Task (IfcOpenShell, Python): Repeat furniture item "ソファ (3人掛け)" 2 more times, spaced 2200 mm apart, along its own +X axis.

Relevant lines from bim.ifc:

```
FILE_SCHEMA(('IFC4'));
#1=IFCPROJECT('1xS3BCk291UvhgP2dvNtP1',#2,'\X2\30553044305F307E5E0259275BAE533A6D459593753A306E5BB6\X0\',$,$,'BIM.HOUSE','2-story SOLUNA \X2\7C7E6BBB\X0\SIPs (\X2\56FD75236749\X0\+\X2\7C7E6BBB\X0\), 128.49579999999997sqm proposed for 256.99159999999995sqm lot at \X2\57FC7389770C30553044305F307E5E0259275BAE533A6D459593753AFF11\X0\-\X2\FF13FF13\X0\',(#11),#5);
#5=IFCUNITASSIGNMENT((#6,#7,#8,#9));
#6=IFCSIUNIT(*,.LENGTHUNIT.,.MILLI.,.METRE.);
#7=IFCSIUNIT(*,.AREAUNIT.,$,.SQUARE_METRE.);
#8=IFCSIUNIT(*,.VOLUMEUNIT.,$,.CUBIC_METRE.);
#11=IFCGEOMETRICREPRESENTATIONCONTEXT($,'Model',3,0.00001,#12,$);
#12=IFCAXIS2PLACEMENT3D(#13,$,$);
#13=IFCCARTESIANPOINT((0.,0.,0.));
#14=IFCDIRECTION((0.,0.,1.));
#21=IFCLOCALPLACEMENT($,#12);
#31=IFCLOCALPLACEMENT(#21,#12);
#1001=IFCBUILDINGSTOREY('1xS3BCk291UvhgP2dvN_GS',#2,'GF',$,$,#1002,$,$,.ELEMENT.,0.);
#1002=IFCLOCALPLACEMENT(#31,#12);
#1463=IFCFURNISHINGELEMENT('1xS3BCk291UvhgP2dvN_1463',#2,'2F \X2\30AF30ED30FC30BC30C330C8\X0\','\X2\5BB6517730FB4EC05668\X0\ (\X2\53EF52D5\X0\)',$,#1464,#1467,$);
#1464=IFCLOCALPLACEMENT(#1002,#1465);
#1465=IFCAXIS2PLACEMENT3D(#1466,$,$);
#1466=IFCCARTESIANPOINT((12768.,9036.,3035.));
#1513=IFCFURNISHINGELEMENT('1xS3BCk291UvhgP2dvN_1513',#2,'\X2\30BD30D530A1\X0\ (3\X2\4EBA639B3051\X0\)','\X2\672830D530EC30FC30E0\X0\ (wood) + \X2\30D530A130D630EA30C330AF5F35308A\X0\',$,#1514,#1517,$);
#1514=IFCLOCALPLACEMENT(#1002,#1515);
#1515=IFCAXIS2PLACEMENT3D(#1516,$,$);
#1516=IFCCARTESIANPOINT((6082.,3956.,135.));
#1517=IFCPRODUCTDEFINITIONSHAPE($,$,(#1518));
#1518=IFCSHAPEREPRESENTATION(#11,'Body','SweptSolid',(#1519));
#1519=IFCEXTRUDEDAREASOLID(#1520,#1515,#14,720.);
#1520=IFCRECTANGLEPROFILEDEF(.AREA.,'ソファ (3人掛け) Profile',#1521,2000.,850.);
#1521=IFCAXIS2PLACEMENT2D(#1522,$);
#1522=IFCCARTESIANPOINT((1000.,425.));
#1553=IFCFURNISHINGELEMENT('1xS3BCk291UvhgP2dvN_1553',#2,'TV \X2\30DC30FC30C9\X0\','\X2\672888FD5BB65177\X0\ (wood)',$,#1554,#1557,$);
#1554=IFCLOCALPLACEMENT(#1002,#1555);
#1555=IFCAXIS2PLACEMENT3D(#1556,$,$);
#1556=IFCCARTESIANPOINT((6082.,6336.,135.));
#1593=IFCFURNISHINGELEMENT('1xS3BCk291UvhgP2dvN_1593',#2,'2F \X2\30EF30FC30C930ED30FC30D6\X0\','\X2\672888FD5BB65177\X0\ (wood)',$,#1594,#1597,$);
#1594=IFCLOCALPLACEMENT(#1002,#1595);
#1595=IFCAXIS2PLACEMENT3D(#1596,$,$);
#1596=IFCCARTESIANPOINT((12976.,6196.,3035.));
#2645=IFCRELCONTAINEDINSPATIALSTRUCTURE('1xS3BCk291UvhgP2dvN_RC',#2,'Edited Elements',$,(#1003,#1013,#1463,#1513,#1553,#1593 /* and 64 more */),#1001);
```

```python
import ifcopenshell
import ifcopenshell.api.geometry
import ifcopenshell.api.root
import ifcopenshell.util.element
import ifcopenshell.util.placement
import ifcopenshell.util.unit

model = ifcopenshell.open("bim.ifc")
unit_scale = ifcopenshell.util.unit.calculate_unit_scale(model)


def reuse_history(source, copy):
    """copy_class also copies each property set's owner history, people and application; keep the originals."""
    for rel in copy.IsDefinedBy:
        if rel.is_a("IfcRelDefinesByProperties") and (history := rel.RelatingPropertyDefinition.OwnerHistory):
            rel.RelatingPropertyDefinition.OwnerHistory = source.OwnerHistory
            ifcopenshell.util.element.remove_deep2(model, history)


source = model.by_id(1513)
base = ifcopenshell.util.placement.get_local_placement(source.ObjectPlacement)
step = base[:3, 0] * 2.2 / unit_scale

for i in range(1, 3):
    copy = ifcopenshell.api.root.copy_class(model, product=source)
    copy.Representation = ifcopenshell.util.element.copy_deep(
        model, source.Representation, exclude=["IfcGeometricRepresentationContext", "IfcRepresentationMap"]
    )
    reuse_history(source, copy)
    matrix = base.copy()
    matrix[:3, 3] += i * step
    print("added at", matrix[:3, 3].round(3) + 0.0)
    ifcopenshell.api.geometry.edit_object_placement(model, product=copy, matrix=matrix, is_si=False)

model.write("bim_edited.ifc")
```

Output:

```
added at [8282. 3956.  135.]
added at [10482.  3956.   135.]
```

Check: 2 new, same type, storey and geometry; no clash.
